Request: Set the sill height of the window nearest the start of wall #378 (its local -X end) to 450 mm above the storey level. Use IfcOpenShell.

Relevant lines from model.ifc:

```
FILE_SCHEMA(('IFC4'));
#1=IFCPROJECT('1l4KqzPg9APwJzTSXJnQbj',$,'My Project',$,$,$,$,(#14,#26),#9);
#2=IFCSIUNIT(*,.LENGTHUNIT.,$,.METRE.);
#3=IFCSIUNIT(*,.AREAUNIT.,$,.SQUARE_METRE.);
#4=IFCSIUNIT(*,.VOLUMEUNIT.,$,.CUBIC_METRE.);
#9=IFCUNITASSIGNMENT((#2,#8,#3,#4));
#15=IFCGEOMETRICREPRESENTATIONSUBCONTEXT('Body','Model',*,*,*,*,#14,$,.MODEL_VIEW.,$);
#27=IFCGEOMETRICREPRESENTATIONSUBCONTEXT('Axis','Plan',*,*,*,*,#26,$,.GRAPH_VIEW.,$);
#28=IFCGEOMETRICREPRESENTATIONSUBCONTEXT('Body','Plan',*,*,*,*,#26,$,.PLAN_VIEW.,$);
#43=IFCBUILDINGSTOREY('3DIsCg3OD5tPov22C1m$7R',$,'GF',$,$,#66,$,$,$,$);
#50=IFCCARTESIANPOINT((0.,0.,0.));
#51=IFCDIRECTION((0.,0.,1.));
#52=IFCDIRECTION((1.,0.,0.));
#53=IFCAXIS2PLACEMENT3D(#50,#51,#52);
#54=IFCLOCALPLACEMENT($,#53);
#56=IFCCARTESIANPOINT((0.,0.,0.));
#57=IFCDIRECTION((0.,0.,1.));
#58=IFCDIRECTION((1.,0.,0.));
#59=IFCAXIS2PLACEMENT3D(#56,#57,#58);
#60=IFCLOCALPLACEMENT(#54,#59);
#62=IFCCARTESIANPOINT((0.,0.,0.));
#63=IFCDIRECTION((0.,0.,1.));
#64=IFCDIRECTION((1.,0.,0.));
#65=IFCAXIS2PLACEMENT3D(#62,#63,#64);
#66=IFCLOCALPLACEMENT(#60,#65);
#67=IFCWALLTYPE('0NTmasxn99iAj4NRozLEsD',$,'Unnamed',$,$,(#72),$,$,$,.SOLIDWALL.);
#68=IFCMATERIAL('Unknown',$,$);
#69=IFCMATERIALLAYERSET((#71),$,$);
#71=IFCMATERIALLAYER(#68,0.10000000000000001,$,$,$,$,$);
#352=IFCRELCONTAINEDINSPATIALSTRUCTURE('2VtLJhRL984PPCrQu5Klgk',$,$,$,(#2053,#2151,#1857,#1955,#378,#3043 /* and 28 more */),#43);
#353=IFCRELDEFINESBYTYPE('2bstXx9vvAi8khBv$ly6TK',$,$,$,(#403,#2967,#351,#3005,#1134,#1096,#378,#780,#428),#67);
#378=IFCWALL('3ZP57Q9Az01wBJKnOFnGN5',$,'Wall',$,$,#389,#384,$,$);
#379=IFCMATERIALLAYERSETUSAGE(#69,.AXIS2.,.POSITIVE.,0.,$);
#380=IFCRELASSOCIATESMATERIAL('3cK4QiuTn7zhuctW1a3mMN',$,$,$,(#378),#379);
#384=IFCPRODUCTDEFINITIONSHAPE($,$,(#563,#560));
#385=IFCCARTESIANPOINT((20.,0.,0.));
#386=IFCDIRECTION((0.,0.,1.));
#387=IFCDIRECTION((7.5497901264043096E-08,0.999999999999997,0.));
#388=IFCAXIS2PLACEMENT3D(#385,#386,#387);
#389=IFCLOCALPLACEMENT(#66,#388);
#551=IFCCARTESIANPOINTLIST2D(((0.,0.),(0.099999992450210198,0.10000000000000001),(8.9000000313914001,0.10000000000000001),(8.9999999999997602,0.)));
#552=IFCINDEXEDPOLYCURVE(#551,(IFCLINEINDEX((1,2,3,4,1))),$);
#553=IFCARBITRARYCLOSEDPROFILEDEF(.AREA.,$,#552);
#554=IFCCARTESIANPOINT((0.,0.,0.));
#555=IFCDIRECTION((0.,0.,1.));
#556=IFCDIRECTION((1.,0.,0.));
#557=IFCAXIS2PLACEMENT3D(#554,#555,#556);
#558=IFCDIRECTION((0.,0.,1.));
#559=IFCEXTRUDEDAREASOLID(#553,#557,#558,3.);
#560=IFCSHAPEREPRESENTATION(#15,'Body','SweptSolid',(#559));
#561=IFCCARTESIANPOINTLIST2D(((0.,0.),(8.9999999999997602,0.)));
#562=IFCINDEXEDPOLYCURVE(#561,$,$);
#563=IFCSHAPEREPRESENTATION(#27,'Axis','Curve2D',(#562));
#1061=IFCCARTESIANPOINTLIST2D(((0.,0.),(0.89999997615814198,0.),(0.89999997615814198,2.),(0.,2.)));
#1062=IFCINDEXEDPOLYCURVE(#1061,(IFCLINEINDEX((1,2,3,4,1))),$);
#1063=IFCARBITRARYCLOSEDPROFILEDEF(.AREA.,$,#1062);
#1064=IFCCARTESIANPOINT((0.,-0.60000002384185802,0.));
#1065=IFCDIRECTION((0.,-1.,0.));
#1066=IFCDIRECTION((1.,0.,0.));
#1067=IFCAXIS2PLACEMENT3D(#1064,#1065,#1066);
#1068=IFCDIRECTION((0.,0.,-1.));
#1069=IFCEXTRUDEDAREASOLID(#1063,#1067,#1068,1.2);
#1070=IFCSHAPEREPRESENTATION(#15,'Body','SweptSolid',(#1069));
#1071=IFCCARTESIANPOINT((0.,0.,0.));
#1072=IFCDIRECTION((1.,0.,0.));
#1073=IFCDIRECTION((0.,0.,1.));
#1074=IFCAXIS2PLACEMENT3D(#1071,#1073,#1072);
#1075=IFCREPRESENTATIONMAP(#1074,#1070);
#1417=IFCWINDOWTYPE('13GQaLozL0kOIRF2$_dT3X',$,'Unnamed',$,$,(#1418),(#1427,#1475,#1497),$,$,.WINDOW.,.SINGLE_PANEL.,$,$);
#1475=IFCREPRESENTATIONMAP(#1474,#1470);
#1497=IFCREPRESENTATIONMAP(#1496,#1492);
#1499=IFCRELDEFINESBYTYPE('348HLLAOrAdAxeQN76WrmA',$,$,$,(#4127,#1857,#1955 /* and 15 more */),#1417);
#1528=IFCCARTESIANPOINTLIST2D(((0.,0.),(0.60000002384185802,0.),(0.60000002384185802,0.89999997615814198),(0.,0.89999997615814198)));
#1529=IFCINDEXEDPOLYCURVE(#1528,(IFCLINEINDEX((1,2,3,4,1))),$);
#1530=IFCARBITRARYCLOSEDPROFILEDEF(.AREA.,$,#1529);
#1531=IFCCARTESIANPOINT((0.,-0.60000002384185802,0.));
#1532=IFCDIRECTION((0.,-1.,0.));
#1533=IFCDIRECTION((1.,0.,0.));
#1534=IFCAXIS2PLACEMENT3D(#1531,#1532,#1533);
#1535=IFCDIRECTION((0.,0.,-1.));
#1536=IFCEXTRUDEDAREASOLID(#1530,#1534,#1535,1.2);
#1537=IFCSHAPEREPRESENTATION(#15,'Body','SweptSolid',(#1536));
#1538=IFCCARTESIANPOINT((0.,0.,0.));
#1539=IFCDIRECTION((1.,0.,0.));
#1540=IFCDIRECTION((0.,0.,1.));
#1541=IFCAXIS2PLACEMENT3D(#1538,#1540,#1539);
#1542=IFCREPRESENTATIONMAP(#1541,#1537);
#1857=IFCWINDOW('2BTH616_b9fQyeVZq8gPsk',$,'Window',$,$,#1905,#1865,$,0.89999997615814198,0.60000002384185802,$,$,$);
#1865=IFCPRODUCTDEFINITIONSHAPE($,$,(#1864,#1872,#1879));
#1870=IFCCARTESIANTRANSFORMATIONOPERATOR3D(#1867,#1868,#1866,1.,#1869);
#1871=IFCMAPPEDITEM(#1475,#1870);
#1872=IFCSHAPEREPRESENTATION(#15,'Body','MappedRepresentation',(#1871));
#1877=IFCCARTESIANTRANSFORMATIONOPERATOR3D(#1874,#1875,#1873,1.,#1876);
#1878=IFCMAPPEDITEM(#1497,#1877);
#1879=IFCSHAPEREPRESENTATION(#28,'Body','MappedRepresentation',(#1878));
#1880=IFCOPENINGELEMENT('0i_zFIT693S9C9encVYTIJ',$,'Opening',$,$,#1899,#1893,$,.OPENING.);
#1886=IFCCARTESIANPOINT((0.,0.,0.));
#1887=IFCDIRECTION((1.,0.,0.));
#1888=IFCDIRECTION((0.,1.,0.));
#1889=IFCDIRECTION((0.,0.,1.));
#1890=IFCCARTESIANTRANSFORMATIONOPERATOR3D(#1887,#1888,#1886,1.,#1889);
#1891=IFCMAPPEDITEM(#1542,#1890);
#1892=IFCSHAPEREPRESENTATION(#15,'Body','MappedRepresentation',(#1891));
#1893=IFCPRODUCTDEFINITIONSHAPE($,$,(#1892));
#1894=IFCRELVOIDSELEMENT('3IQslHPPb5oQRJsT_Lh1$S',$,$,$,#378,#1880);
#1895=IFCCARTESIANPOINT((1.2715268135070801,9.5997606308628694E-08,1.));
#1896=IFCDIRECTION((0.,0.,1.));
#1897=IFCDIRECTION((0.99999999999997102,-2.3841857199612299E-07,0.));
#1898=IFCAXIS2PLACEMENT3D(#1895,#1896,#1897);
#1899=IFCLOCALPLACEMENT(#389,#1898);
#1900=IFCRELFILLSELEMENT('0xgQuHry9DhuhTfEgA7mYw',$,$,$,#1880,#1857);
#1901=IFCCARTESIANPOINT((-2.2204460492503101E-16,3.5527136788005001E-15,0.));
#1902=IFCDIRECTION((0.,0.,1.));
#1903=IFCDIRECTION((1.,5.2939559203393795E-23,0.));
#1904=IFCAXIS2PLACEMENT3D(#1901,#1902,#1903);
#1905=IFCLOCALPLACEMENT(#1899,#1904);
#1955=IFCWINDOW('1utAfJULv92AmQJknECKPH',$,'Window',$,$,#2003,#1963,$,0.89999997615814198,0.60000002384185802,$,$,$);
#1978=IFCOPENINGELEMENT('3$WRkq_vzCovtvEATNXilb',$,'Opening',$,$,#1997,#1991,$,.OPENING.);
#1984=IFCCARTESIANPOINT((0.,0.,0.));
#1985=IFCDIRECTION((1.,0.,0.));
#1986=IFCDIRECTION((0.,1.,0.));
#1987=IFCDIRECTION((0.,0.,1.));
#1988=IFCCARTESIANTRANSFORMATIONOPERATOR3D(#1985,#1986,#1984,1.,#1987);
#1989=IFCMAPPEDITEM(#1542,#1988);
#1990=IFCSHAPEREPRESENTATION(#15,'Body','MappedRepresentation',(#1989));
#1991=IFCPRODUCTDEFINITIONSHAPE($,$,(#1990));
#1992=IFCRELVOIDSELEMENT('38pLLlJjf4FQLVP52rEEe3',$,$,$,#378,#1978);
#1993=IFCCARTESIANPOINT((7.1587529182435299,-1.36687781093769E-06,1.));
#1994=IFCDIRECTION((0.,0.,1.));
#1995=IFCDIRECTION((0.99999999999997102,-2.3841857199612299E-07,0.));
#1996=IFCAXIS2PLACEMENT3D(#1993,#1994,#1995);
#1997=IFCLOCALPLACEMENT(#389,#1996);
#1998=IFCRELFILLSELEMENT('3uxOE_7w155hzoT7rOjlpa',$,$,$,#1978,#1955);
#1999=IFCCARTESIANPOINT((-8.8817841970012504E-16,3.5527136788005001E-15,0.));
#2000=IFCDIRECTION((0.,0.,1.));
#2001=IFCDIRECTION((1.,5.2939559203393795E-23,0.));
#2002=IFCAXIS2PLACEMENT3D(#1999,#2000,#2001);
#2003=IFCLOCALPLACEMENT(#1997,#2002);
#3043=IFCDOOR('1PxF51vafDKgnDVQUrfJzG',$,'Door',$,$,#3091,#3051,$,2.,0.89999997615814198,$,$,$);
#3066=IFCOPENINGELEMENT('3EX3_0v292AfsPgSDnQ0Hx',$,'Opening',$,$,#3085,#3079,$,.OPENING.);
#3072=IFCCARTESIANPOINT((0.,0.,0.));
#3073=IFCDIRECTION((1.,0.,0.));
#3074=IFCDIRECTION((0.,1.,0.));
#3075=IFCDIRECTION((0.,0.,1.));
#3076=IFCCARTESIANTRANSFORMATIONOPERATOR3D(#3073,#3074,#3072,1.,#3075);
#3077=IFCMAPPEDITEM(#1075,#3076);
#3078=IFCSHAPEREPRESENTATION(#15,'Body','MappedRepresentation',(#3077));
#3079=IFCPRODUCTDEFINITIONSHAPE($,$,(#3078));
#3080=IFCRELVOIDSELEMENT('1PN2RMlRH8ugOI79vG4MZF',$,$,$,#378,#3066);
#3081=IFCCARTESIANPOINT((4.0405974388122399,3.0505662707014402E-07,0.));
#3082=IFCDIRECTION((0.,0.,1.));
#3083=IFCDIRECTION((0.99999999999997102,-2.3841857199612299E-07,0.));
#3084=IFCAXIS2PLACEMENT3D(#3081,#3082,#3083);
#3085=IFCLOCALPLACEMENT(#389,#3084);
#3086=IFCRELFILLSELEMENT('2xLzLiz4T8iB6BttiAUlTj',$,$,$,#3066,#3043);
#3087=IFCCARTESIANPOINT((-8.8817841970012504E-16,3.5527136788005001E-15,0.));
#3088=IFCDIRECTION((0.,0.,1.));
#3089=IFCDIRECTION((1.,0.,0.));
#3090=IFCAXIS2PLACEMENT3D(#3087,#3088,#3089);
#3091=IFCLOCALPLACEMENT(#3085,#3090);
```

```python
import numpy as np
import ifcopenshell
import ifcopenshell.api.geometry
import ifcopenshell.geom
import ifcopenshell.util.element
import ifcopenshell.util.placement
import ifcopenshell.util.shape
import ifcopenshell.util.unit

model = ifcopenshell.open("model.ifc")
unit_scale = ifcopenshell.util.unit.calculate_unit_scale(model)

window = model.by_guid("2BTH616_b9fQyeVZq8gPsk")
opening = window.FillsVoids[0].RelatingOpeningElement
storey = ifcopenshell.util.element.get_container(window, ifc_class="IfcBuildingStorey")
level = ifcopenshell.util.placement.get_local_placement(storey.ObjectPlacement)[2, 3]

# The opening's origin need not be at the sill, so measure its lowest point.
shape = ifcopenshell.geom.create_shape(ifcopenshell.geom.settings(), opening)
bottom = ifcopenshell.util.shape.get_shape_bottom_elevation(shape, shape.geometry) / unit_scale
dz = level + 0.45 - bottom

shift = np.array([0.0, 0.0, dz])
# The window is placed relative to its opening, so it follows when the opening moves.
matrix = ifcopenshell.util.placement.get_local_placement(opening.ObjectPlacement)
matrix[:3, 3] += shift
ifcopenshell.api.geometry.edit_object_placement(
    model, product=opening, matrix=matrix, is_si=False, should_transform_children=True
)

print(f"moved by {dz * unit_scale:+.3f} m")

model.write("model_v2.ifc")
```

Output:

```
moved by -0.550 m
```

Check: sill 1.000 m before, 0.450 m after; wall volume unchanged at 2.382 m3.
